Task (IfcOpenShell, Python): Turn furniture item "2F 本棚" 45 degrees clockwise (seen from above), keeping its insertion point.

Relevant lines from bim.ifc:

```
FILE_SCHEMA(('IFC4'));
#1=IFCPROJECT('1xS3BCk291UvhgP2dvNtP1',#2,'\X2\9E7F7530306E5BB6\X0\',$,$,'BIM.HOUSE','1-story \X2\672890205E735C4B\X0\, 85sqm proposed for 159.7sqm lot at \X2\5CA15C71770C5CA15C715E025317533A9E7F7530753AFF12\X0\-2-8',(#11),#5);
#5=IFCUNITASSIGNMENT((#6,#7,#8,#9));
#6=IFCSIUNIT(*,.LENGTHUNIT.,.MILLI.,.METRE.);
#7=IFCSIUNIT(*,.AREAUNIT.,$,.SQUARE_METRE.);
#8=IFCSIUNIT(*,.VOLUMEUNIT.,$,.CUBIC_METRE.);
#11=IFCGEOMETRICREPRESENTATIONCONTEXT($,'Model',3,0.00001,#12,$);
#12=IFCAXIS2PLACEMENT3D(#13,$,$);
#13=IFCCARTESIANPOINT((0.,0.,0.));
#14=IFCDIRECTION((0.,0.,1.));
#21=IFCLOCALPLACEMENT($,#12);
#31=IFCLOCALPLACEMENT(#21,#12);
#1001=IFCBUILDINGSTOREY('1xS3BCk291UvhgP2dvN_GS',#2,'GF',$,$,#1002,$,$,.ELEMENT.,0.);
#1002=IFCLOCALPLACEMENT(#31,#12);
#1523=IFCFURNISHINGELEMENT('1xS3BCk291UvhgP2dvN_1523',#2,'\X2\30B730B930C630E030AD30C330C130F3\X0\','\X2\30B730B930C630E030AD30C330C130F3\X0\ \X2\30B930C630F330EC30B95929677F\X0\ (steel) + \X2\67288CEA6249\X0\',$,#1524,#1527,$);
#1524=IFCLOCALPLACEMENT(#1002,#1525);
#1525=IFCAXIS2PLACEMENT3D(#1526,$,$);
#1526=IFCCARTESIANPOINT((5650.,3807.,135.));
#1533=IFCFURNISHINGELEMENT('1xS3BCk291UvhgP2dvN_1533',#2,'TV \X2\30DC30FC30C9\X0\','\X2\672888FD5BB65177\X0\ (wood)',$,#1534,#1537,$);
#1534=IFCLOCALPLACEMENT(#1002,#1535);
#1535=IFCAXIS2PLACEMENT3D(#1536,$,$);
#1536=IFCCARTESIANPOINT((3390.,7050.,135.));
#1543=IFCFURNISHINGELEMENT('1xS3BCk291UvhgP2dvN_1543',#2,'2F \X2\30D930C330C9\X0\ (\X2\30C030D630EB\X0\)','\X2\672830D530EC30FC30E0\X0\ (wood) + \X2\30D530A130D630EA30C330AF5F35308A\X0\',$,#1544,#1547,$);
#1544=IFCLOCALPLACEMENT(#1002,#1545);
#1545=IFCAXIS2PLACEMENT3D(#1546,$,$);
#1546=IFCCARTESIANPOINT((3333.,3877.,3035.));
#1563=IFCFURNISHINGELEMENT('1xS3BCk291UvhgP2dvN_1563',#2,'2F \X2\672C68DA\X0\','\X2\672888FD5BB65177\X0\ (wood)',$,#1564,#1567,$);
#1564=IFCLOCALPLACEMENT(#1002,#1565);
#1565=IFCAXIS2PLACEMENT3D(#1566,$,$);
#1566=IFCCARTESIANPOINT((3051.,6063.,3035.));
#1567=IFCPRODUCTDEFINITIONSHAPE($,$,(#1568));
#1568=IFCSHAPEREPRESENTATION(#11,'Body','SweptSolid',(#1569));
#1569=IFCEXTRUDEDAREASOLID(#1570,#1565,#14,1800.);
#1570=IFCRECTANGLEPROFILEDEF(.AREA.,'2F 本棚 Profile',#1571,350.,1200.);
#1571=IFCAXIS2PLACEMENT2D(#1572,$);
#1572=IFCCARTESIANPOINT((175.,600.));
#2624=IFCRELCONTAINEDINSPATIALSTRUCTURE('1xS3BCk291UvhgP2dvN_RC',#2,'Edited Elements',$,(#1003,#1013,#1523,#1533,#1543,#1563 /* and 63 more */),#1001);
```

```python
import ifcopenshell
import ifcopenshell.api.geometry
import ifcopenshell.util.placement

model = ifcopenshell.open("bim.ifc")

item = model.by_id(1563)
matrix = ifcopenshell.util.placement.get_local_placement(item.ObjectPlacement)
matrix = matrix @ ifcopenshell.util.placement.rotation(-45, "Z")
ifcopenshell.api.geometry.edit_object_placement(model, product=item, matrix=matrix, is_si=False)

print(ifcopenshell.util.placement.get_local_placement(item.ObjectPlacement).round(3) + 0.0)

model.write("bim_v2.ifc")
```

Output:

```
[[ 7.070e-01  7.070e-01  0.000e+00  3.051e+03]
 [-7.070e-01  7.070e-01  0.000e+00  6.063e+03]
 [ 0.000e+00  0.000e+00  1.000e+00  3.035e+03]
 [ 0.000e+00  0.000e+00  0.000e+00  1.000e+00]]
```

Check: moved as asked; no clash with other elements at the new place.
